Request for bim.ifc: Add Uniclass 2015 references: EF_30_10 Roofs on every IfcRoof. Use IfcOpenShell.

First a look at what the model holds.

```python
import ifcopenshell

model = ifcopenshell.open("bim.ifc")
print(model.schema)
print("classifications:", [c.Name for c in model.by_type("IfcClassification")])
for ifc_class in ("IfcDoor", "IfcRoof", "IfcStair", "IfcWall", "IfcWindow"):
    print(ifc_class, len(model.by_type(ifc_class)))
```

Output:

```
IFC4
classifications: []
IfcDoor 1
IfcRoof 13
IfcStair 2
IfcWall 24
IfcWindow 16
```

```python
import ifcopenshell
import ifcopenshell.api.classification

model = ifcopenshell.open("bim.ifc")

system = ifcopenshell.api.classification.add_classification(model, classification="Uniclass 2015")

codes = {
    "IfcRoof": ("EF_30_10", "Roofs"),
}
for ifc_class, (code, name) in codes.items():
    products = model.by_type(ifc_class)
    ifcopenshell.api.classification.add_reference(
        model, products=products, classification=system, identification=code, name=name
    )
    print(code, len(products))

model.write("bim-out.ifc")
```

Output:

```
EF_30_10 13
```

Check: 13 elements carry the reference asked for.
